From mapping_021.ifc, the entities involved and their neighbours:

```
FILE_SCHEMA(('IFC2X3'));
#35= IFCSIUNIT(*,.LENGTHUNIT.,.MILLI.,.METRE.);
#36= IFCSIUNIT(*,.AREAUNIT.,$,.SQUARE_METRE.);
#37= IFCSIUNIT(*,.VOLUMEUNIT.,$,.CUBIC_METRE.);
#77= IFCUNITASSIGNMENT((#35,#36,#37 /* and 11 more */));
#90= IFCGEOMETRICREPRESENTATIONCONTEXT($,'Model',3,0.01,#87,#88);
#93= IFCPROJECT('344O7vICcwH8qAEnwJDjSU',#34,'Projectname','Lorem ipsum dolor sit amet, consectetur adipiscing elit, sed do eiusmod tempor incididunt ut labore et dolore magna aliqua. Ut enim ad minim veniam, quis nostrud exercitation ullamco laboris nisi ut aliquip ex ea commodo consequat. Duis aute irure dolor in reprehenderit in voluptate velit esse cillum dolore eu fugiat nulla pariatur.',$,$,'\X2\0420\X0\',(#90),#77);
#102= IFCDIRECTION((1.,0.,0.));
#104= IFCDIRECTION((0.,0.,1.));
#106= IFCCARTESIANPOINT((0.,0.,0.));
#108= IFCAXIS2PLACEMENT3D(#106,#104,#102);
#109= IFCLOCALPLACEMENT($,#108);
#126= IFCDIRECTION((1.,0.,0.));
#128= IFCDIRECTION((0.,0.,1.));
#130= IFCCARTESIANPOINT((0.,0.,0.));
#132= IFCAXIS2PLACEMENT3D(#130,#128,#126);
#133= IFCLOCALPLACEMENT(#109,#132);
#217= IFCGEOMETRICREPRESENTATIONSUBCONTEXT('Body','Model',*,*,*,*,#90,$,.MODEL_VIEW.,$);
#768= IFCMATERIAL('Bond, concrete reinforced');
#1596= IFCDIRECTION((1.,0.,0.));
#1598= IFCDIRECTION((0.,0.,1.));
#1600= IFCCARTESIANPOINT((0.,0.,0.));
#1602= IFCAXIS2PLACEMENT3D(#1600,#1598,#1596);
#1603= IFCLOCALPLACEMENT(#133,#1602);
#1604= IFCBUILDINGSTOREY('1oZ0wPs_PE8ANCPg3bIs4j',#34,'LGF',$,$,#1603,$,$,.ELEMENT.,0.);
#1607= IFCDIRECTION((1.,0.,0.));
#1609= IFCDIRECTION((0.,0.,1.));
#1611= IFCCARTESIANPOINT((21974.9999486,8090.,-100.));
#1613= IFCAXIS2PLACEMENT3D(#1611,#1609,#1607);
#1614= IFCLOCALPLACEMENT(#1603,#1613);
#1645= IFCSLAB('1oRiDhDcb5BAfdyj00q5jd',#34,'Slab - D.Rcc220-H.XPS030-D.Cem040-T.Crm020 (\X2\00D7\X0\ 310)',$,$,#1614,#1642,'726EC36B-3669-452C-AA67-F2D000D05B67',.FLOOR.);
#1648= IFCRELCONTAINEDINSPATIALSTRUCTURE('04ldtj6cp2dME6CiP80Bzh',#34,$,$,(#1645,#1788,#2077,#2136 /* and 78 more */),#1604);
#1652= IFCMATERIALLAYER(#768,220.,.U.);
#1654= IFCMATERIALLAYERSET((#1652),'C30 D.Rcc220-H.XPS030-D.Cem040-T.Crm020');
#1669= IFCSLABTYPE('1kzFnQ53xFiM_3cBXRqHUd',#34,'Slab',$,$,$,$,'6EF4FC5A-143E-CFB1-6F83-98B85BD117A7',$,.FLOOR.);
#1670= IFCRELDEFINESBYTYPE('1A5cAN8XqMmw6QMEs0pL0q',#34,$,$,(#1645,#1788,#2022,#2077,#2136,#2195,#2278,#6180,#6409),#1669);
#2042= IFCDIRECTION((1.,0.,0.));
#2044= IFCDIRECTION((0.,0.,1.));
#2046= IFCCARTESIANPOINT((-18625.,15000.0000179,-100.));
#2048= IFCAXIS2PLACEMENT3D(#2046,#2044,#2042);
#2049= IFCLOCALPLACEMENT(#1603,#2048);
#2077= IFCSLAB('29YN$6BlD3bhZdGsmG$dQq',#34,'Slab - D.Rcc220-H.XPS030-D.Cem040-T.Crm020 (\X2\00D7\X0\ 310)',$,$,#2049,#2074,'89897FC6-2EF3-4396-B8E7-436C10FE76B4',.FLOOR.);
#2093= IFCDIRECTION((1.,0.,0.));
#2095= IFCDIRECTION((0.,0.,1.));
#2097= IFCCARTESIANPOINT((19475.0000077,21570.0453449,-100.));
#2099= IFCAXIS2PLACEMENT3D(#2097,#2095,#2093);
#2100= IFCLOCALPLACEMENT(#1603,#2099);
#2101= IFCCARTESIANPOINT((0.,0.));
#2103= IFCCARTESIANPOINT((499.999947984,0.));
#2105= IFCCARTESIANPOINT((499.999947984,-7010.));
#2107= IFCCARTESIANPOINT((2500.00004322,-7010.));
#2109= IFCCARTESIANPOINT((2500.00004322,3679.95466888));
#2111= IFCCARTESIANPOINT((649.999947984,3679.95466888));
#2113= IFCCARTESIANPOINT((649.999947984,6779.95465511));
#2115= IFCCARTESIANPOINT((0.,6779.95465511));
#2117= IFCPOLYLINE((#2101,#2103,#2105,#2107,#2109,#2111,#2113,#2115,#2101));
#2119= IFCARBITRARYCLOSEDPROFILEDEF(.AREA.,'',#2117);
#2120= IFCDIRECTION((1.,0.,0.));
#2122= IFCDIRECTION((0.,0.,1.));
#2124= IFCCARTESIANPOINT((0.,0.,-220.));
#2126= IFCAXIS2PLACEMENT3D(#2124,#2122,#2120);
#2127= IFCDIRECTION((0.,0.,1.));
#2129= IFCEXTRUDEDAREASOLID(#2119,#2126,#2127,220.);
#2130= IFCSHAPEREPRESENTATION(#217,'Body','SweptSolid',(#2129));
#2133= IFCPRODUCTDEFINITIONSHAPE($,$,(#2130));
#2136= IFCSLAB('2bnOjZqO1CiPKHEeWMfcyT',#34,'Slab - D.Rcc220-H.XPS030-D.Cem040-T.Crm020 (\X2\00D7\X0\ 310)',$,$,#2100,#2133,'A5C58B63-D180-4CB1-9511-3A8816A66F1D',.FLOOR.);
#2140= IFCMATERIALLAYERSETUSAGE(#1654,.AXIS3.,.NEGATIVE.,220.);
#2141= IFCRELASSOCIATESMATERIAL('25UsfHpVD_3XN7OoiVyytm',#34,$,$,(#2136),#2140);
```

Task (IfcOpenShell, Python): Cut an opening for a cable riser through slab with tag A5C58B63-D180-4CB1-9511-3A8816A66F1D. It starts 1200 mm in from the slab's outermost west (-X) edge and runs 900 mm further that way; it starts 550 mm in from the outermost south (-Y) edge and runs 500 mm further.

```python
import numpy as np
import ifcopenshell
import ifcopenshell.api.feature
import ifcopenshell.api.geometry
import ifcopenshell.api.root
import ifcopenshell.geom
import ifcopenshell.util.placement
import ifcopenshell.util.representation
import ifcopenshell.util.shape
import ifcopenshell.util.unit

model = ifcopenshell.open("mapping_021.ifc")
unit_scale = ifcopenshell.util.unit.calculate_unit_scale(model)
settings = ifcopenshell.geom.settings()


def volume(element):
    """Net volume in cubic metres, openings subtracted."""
    shape = ifcopenshell.geom.create_shape(settings, element)
    return ifcopenshell.util.shape.get_volume(shape.geometry)


slab = model.by_guid("2bnOjZqO1CiPKHEeWMfcyT")
before = volume(slab)

# Extent in the slab's own axes, in metres. The edges named are its -X and -Y sides.
slab_shape = ifcopenshell.geom.create_shape(settings, slab)
vertices = ifcopenshell.util.shape.get_vertices(slab_shape.geometry)
x_min, y_min, bottom = vertices.min(axis=0)
top = vertices[:, 2].max()

opening = ifcopenshell.api.root.create_entity(model, ifc_class="IfcOpeningElement", name="Cable riser opening")
context = ifcopenshell.util.representation.get_context(model, "Model", "Body", "MODEL_VIEW")
width, depth = 0.9, 0.5
outline = [(0.0, 0.0), (width, 0.0), (width, depth), (0.0, depth), (0.0, 0.0)]
# Overshoot both faces by 50 mm so the cut is clean.
shape = ifcopenshell.api.geometry.add_slab_representation(
    model, context=context, depth=top - bottom + 0.1, polyline=outline
)
ifcopenshell.api.geometry.assign_representation(model, product=opening, representation=shape)

matrix = ifcopenshell.util.placement.get_local_placement(slab.ObjectPlacement)
matrix[:, 3] = matrix @ np.append(np.array([x_min + 1.2, y_min + 0.55, bottom - 0.05]) / unit_scale, 1.0)
ifcopenshell.api.geometry.edit_object_placement(model, product=opening, matrix=matrix, is_si=False)
ifcopenshell.api.feature.add_feature(model, feature=opening, element=slab)

after = volume(slab)

print(f"slab volume {before:.3f} -> {after:.3f} m3")

model.write("mapping_021-out.ifc")
```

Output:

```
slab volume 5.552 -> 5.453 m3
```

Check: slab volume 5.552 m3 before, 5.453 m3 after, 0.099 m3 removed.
